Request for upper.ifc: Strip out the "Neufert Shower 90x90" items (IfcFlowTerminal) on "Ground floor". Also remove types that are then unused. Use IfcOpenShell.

First a look at what the model holds.

```python
import ifcopenshell
import ifcopenshell.util.element

model = ifcopenshell.open("upper.ifc")
print(model.schema)
storey = next(s for s in model.by_type("IfcBuildingStorey") if s.Name == "Ground floor")
terminals = [e for e in ifcopenshell.util.element.get_decomposition(storey) if e.is_a("IfcFlowTerminal")]
seen = {}
for e in terminals:
    element_type = ifcopenshell.util.element.get_type(e)
    name = element_type.Name if element_type not in (None, e) else None
    seen[name] = seen.get(name, 0) + 1
for name, count in sorted(seen.items(), key=str):
    print(count, "x", name)
```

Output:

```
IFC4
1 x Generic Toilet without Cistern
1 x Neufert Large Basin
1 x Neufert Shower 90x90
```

```python
import ifcopenshell
import ifcopenshell.api.root
import ifcopenshell.util.element

model = ifcopenshell.open("upper.ifc")

storey = next(s for s in model.by_type("IfcBuildingStorey") if s.Name == "Ground floor")
terminals = [e for e in ifcopenshell.util.element.get_decomposition(storey) if e.is_a("IfcFlowTerminal")]
targets = [e for e in terminals if (t := ifcopenshell.util.element.get_type(e)) not in (None, e) and t.Name == "Neufert Shower 90x90"]
types = {ifcopenshell.util.element.get_type(e) for e in targets} - {None, *targets}

for e in targets:
    ifcopenshell.api.root.remove_product(model, product=e)
print(len(targets), "removed")

unused = [t for t in types if not ifcopenshell.util.element.get_types(t)]
for t in unused:
    ifcopenshell.api.root.remove_product(model, product=t)
print(len(unused), "unused types removed")

model.write("upper-out.ifc")
```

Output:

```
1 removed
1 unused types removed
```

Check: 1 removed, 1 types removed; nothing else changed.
